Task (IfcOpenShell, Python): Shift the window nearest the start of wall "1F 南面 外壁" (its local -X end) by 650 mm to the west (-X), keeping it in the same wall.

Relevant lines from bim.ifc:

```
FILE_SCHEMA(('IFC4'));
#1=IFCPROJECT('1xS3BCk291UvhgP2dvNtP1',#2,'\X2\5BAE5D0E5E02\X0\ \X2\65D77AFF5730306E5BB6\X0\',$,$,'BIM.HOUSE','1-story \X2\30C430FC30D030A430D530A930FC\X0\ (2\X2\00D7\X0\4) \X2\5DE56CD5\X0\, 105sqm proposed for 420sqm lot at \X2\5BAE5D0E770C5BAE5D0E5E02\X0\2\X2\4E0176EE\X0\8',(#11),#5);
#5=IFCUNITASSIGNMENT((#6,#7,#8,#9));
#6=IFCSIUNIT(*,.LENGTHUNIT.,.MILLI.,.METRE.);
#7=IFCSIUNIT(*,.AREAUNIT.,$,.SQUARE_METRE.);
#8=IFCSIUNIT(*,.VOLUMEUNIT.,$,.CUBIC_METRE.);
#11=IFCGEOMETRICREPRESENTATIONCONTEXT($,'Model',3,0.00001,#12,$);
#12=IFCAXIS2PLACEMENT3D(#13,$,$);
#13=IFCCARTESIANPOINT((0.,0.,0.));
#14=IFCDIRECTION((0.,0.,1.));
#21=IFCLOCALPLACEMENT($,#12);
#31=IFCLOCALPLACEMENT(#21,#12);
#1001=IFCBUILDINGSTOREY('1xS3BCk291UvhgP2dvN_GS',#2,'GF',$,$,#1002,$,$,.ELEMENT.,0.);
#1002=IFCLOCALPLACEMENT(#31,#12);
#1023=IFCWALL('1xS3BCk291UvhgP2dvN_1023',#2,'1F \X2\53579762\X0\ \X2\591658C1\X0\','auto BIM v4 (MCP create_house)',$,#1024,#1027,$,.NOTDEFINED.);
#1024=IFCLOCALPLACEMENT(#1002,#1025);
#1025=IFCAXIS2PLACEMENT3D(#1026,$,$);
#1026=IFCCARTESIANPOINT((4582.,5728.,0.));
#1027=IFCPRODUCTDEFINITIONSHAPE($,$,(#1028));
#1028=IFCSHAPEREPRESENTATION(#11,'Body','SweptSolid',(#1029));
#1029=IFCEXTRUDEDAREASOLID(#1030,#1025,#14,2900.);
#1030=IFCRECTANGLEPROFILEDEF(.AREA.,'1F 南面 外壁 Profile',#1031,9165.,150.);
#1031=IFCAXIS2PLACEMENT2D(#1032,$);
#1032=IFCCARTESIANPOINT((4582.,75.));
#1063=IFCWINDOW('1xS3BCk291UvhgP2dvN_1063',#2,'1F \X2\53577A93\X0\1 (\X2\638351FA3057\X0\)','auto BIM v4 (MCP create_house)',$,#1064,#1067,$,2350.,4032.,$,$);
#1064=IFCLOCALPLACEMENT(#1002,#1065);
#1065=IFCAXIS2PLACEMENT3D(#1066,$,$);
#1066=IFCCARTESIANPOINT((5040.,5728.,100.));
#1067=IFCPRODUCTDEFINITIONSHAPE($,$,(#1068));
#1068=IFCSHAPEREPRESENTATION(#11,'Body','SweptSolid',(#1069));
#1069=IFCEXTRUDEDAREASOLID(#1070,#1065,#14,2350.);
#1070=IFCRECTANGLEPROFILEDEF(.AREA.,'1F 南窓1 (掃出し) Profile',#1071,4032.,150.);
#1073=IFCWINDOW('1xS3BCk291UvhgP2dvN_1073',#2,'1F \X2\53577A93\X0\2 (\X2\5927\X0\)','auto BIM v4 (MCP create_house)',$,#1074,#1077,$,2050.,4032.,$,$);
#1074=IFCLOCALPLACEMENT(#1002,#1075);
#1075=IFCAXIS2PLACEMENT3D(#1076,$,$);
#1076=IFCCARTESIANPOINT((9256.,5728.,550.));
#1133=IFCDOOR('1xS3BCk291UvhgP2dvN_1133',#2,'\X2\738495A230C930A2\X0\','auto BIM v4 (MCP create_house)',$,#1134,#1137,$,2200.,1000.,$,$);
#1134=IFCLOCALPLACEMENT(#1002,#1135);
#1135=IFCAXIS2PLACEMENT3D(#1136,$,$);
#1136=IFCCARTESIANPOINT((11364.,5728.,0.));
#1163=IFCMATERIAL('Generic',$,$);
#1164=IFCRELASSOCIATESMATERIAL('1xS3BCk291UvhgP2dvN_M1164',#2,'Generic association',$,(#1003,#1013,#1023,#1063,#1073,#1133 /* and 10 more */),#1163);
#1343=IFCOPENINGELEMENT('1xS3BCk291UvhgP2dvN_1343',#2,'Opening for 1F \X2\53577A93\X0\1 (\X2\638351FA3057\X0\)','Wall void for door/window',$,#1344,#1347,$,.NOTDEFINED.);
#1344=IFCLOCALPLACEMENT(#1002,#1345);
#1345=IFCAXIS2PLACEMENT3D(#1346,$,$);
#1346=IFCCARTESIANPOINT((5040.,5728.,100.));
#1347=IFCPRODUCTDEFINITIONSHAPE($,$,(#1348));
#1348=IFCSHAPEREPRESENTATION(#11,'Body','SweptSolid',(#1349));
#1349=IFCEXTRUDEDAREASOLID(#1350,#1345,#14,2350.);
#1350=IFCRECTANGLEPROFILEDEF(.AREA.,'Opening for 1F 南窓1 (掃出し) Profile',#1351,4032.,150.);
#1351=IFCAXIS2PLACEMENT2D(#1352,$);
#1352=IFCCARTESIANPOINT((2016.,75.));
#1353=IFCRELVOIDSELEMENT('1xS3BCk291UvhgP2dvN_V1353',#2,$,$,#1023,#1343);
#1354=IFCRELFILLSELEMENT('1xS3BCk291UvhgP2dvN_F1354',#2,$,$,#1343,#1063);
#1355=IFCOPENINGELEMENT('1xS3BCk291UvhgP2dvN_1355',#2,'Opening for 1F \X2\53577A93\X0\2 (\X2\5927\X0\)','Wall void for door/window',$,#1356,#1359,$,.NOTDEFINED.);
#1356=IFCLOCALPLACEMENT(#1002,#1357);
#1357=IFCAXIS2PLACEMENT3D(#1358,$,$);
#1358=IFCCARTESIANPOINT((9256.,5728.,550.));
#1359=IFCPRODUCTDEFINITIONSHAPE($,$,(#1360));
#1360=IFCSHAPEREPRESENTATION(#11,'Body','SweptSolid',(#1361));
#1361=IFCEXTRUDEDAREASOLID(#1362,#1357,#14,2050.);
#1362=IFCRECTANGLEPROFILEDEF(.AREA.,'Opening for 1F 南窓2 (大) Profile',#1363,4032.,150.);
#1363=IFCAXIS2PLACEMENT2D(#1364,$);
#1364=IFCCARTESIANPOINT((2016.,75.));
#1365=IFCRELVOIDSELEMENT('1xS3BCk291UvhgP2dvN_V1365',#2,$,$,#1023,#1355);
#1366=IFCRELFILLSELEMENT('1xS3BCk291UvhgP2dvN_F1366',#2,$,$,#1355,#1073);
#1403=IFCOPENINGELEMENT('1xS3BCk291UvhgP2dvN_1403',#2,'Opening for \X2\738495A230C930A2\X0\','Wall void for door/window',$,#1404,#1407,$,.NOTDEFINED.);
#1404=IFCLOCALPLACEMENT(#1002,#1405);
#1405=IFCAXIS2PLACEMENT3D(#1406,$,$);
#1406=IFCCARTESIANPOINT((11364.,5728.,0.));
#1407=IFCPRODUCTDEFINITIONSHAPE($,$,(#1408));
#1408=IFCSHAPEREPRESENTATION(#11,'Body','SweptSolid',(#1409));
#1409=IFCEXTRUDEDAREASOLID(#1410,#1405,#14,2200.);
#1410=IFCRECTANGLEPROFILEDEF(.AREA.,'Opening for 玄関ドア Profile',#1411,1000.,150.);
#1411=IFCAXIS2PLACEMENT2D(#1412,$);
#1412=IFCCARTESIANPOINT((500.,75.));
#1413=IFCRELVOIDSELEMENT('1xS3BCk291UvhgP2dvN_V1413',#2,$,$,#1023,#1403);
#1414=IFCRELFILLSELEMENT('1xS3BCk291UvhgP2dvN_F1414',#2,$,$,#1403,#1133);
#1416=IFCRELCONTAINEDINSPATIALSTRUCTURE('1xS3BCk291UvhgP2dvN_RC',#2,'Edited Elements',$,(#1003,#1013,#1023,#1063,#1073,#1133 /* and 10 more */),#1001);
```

```python
import ifcopenshell
import ifcopenshell.api.geometry
import ifcopenshell.util.placement

model = ifcopenshell.open("bim.ifc")

window = model.by_guid("1xS3BCk291UvhgP2dvN_1063")
opening = window.FillsVoids[0].RelatingOpeningElement
wall = opening.VoidsElements[0].RelatingBuildingElement

wall_matrix = ifcopenshell.util.placement.get_local_placement(wall.ObjectPlacement)
shift = wall_matrix[:3, 0] * -650.0
before = ifcopenshell.util.placement.get_local_placement(window.ObjectPlacement)[:3, 3].copy()

# The window is not placed relative to its opening, so move both.
for product in (opening, window):
    matrix = ifcopenshell.util.placement.get_local_placement(product.ObjectPlacement)
    matrix[:3, 3] += shift
    ifcopenshell.api.geometry.edit_object_placement(model, product=product, matrix=matrix, is_si=False)

after = ifcopenshell.util.placement.get_local_placement(window.ObjectPlacement)[:3, 3]
print("window moved by", (after - before).round(3) + 0.0)

model.write("bim_v2.ifc")
```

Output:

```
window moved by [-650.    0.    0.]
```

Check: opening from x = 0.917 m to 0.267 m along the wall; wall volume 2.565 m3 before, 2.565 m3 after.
